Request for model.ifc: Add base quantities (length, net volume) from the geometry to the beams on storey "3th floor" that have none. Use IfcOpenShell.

First a look at what the model holds.

```python
import ifcopenshell
import ifcopenshell.util.element
import ifcopenshell.util.unit

model = ifcopenshell.open("model.ifc")
print(model.schema)
for unit_type in ("LENGTHUNIT", "AREAUNIT", "VOLUMEUNIT"):
    print(unit_type, ifcopenshell.util.unit.calculate_unit_scale(model, unit_type))
storey = next(s for s in model.by_type("IfcBuildingStorey") if s.Name == "3th floor")
beams = [e for e in ifcopenshell.util.element.get_decomposition(storey) if e.is_a("IfcBeam")]
for e in sorted(beams, key=lambda e: e.id()):
    print(e.id(), e.is_a(), e.Name, list(ifcopenshell.util.element.get_psets(e, qtos_only=True)), sep=" | ")
```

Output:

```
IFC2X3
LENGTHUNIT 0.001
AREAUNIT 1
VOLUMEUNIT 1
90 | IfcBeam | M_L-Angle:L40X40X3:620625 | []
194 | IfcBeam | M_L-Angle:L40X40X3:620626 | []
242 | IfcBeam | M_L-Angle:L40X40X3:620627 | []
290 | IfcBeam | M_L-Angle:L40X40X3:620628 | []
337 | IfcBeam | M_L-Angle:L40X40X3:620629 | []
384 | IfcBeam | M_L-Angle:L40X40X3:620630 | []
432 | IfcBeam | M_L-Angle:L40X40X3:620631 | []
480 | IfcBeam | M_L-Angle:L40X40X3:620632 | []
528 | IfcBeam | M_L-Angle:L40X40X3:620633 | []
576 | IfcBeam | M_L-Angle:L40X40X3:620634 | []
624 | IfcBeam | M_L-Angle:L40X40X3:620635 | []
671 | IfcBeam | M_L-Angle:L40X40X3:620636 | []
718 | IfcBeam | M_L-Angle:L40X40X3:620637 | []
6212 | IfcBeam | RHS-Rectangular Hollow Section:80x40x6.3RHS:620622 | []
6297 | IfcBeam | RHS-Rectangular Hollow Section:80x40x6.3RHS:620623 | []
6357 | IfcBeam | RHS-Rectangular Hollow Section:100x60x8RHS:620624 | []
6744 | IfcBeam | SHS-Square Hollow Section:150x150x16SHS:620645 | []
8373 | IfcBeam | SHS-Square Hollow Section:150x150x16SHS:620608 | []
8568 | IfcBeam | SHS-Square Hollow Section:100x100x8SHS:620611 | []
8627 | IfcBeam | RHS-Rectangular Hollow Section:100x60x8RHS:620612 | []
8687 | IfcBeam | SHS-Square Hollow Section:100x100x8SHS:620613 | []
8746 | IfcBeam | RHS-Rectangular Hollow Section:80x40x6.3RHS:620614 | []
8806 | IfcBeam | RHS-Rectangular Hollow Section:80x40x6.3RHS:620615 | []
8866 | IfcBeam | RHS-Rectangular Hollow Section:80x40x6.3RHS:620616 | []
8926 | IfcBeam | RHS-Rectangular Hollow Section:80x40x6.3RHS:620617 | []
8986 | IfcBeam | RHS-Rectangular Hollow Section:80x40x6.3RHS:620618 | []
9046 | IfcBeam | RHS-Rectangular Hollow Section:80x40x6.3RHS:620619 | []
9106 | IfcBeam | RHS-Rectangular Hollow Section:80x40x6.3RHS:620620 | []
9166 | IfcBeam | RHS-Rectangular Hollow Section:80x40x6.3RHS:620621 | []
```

```python
import ifcopenshell
import ifcopenshell.api.pset
import ifcopenshell.geom
import ifcopenshell.util.element
import ifcopenshell.util.shape
import ifcopenshell.util.unit

model = ifcopenshell.open("model.ifc")
unit_scale = ifcopenshell.util.unit.calculate_unit_scale(model)
volume_scale = ifcopenshell.util.unit.calculate_unit_scale(model, "VOLUMEUNIT")
settings = ifcopenshell.geom.settings()

storey = next(s for s in model.by_type("IfcBuildingStorey") if s.Name == "3th floor")
beams = [e for e in ifcopenshell.util.element.get_decomposition(storey) if e.is_a("IfcBeam")]

for e in sorted(beams, key=lambda e: e.id()):
    if ifcopenshell.util.element.get_psets(e, qtos_only=True, should_inherit=False):
        continue
    # Geometry comes back in metres, in the element's own axes.
    shape = ifcopenshell.geom.create_shape(settings, e)
    values = {
        "Length": ifcopenshell.util.shape.get_max_xyz(shape.geometry) / unit_scale,
        "NetVolume": ifcopenshell.util.shape.get_volume(shape.geometry) / volume_scale,
    }
    qto = ifcopenshell.api.pset.add_qto(model, product=e, name="BaseQuantities")
    ifcopenshell.api.pset.edit_qto(model, qto=qto, properties=values)
    print(e.id(), {k: round(v, 3) for k, v in values.items()})

model.write("model_rev.ifc")
```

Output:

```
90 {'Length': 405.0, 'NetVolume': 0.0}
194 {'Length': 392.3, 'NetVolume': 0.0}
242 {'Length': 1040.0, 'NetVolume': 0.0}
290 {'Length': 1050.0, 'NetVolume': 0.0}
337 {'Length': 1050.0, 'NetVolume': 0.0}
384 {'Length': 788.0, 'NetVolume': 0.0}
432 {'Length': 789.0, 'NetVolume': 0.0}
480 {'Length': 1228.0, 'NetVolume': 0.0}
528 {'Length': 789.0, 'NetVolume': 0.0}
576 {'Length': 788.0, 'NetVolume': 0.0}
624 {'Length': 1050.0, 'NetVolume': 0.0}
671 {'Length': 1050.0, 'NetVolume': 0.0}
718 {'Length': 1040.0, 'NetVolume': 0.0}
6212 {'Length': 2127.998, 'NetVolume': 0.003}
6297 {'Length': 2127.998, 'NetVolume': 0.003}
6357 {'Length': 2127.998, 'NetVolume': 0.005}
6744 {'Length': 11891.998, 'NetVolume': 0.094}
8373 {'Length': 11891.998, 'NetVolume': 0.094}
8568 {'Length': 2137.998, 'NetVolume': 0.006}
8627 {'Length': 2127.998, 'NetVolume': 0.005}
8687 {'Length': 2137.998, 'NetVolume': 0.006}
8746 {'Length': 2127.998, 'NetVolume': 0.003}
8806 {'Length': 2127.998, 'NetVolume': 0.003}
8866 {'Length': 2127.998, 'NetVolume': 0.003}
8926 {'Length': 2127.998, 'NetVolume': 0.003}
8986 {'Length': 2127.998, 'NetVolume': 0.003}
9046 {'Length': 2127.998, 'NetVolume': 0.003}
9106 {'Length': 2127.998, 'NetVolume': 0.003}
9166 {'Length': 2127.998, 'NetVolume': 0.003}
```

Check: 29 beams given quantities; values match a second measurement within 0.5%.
